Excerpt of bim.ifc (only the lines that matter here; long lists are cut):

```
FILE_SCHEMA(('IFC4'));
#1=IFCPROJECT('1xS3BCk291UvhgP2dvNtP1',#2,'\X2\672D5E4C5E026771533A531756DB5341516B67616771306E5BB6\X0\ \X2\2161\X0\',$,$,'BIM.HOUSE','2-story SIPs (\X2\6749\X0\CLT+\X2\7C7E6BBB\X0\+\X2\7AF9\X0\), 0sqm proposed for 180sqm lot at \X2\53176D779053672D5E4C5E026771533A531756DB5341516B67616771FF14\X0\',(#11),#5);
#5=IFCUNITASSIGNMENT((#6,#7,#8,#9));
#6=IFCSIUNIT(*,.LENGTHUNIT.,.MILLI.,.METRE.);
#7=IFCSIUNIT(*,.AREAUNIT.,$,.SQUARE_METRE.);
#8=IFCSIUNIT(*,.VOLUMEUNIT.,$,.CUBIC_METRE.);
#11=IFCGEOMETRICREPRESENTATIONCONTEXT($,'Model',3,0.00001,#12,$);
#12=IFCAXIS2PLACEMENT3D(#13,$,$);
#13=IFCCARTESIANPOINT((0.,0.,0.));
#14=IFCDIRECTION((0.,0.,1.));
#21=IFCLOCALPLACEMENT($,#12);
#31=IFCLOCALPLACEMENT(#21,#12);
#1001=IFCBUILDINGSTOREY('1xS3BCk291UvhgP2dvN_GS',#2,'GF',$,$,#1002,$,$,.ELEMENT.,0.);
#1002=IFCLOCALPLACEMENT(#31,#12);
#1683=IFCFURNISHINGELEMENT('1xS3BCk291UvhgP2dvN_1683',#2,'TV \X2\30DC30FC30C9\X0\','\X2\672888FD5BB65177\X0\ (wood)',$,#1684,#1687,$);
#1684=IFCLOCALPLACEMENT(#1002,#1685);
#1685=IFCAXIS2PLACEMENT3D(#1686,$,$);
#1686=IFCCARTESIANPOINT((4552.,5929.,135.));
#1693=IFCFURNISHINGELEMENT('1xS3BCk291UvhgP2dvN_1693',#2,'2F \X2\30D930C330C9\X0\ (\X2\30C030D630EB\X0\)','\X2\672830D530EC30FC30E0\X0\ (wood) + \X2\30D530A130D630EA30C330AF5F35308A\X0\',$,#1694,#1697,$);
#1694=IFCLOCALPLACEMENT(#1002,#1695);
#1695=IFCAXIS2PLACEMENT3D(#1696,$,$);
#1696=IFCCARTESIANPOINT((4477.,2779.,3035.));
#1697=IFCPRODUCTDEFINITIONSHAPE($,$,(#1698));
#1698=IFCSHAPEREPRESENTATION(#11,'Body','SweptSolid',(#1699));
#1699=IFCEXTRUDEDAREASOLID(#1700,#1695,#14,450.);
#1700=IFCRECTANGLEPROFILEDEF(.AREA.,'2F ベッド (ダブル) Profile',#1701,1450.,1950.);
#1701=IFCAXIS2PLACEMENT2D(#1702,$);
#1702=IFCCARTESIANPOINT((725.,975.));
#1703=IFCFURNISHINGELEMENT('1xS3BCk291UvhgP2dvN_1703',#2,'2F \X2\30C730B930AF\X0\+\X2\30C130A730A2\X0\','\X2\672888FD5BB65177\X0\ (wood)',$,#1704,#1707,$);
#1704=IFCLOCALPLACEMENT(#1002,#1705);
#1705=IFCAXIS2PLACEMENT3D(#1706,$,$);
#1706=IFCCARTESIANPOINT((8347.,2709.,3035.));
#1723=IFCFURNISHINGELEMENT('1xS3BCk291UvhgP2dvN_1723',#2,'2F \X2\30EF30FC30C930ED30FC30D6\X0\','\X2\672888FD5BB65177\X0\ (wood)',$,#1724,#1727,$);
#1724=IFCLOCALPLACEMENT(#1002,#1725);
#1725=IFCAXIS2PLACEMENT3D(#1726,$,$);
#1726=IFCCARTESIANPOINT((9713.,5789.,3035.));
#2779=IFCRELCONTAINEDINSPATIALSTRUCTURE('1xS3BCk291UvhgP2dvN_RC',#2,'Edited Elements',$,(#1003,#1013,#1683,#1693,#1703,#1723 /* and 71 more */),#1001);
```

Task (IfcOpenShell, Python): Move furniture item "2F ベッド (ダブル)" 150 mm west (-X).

```python
import ifcopenshell
import ifcopenshell.api.geometry
import ifcopenshell.util.placement
import ifcopenshell.util.unit

model = ifcopenshell.open("bim.ifc")
unit_scale = ifcopenshell.util.unit.calculate_unit_scale(model)

item = model.by_guid("1xS3BCk291UvhgP2dvN_1693")
matrix = ifcopenshell.util.placement.get_local_placement(item.ObjectPlacement)
matrix[0, 3] -= 0.15 / unit_scale
ifcopenshell.api.geometry.edit_object_placement(model, product=item, matrix=matrix, is_si=False)

print(ifcopenshell.util.placement.get_local_placement(item.ObjectPlacement).round(3) + 0.0)

model.write("bim-out.ifc")
```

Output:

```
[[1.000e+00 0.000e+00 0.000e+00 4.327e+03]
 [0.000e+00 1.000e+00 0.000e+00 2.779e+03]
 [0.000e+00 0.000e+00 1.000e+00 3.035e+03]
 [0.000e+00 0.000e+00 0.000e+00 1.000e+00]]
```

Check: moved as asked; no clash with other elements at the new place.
